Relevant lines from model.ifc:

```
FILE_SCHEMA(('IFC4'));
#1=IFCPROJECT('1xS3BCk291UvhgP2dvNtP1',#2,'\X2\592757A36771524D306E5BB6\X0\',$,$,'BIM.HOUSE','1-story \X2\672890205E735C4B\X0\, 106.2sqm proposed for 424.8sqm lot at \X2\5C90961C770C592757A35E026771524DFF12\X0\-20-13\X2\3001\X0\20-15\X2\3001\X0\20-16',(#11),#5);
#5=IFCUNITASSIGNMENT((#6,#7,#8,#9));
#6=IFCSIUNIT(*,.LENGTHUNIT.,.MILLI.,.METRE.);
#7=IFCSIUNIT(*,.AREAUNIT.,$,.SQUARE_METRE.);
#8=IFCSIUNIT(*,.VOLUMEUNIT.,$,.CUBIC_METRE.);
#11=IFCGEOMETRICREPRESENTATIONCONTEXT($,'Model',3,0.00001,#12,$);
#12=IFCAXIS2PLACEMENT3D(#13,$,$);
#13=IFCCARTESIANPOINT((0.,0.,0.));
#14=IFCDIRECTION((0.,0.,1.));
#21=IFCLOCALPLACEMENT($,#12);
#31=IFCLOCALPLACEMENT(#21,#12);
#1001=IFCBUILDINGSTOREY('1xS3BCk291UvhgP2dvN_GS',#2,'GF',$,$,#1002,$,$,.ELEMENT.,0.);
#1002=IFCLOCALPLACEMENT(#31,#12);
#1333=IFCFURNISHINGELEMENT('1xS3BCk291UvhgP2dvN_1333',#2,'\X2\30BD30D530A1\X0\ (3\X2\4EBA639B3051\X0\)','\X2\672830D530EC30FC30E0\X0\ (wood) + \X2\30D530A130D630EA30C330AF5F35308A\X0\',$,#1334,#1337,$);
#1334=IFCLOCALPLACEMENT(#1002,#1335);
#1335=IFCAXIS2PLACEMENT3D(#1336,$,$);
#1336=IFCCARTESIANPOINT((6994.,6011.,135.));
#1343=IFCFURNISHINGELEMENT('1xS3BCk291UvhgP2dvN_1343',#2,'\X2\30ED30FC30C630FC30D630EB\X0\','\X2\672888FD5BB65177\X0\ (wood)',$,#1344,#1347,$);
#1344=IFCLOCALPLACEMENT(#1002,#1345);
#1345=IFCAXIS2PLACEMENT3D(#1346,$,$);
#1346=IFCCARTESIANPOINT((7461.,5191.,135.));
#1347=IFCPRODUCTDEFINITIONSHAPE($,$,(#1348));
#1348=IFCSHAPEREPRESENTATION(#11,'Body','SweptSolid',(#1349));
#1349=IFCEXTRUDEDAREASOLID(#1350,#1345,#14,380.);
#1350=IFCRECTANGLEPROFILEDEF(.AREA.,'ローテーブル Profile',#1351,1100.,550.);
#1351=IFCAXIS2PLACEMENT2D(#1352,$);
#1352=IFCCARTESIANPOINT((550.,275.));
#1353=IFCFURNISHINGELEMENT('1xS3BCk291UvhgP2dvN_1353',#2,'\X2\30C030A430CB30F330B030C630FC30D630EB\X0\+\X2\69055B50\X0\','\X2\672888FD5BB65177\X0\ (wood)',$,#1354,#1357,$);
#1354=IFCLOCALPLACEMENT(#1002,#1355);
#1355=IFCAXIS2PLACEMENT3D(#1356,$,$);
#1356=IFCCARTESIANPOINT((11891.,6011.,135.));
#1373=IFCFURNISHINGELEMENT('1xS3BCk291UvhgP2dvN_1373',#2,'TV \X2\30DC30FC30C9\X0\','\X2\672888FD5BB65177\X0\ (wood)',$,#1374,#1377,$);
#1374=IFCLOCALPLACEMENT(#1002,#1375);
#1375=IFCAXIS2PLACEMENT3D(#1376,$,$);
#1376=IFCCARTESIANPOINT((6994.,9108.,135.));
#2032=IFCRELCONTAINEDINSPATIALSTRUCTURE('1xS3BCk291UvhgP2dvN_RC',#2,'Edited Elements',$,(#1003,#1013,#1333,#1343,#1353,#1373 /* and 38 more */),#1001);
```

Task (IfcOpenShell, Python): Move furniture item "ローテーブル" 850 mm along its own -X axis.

```python
import ifcopenshell
import ifcopenshell.api.geometry
import ifcopenshell.util.placement
import ifcopenshell.util.unit

model = ifcopenshell.open("model.ifc")
unit_scale = ifcopenshell.util.unit.calculate_unit_scale(model)

item = model.by_guid("1xS3BCk291UvhgP2dvN_1343")
matrix = ifcopenshell.util.placement.get_local_placement(item.ObjectPlacement)
matrix[:3, 3] -= matrix[:3, 0] * 0.85 / unit_scale
ifcopenshell.api.geometry.edit_object_placement(model, product=item, matrix=matrix, is_si=False)

print(ifcopenshell.util.placement.get_local_placement(item.ObjectPlacement).round(3) + 0.0)

model.write("model_v2.ifc")
```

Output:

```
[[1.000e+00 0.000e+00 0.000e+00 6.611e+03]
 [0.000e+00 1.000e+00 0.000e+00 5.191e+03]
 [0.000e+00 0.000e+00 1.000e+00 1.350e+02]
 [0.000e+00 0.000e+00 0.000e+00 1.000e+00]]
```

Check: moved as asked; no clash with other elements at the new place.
